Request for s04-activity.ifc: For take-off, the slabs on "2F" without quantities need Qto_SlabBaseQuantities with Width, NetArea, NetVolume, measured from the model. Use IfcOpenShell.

First a look at what the model holds.

```python
import ifcopenshell
import ifcopenshell.util.element
import ifcopenshell.util.unit

model = ifcopenshell.open("s04-activity.ifc")
print(model.schema)
for unit_type in ("LENGTHUNIT", "AREAUNIT", "VOLUMEUNIT"):
    print(unit_type, ifcopenshell.util.unit.calculate_unit_scale(model, unit_type))
storey = next(s for s in model.by_type("IfcBuildingStorey") if s.Name == "2F")
slabs = [e for e in ifcopenshell.util.element.get_decomposition(storey) if e.is_a("IfcSlab")]
for e in sorted(slabs, key=lambda e: e.id()):
    print(e.id(), e.is_a(), e.Name, list(ifcopenshell.util.element.get_psets(e, qtos_only=True)), sep=" | ")
```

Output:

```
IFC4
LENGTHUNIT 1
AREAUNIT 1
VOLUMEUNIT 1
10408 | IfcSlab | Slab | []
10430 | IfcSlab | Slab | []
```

```python
import ifcopenshell
import ifcopenshell.api.pset
import ifcopenshell.geom
import ifcopenshell.util.element
import ifcopenshell.util.shape
import ifcopenshell.util.unit

model = ifcopenshell.open("s04-activity.ifc")
unit_scale = ifcopenshell.util.unit.calculate_unit_scale(model)
area_scale = ifcopenshell.util.unit.calculate_unit_scale(model, "AREAUNIT")
volume_scale = ifcopenshell.util.unit.calculate_unit_scale(model, "VOLUMEUNIT")
settings = ifcopenshell.geom.settings()

storey = next(s for s in model.by_type("IfcBuildingStorey") if s.Name == "2F")
slabs = [e for e in ifcopenshell.util.element.get_decomposition(storey) if e.is_a("IfcSlab")]

for e in sorted(slabs, key=lambda e: e.id()):
    if ifcopenshell.util.element.get_psets(e, qtos_only=True, should_inherit=False):
        continue
    # Geometry comes back in metres, in the element's own axes.
    shape = ifcopenshell.geom.create_shape(settings, e)
    values = {
        "Width": ifcopenshell.util.shape.get_z(shape.geometry) / unit_scale,
        "NetArea": ifcopenshell.util.shape.get_footprint_area(shape.geometry) / area_scale,
        "NetVolume": ifcopenshell.util.shape.get_volume(shape.geometry) / volume_scale,
    }
    qto = ifcopenshell.api.pset.add_qto(model, product=e, name="Qto_SlabBaseQuantities")
    ifcopenshell.api.pset.edit_qto(model, qto=qto, properties=values)
    print(e.id(), {k: round(v, 3) for k, v in values.items()})

model.write("s04-activity_rev.ifc")
```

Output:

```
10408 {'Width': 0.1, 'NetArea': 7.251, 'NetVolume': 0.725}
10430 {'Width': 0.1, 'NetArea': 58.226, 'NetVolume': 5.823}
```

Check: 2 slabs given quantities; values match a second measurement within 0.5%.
